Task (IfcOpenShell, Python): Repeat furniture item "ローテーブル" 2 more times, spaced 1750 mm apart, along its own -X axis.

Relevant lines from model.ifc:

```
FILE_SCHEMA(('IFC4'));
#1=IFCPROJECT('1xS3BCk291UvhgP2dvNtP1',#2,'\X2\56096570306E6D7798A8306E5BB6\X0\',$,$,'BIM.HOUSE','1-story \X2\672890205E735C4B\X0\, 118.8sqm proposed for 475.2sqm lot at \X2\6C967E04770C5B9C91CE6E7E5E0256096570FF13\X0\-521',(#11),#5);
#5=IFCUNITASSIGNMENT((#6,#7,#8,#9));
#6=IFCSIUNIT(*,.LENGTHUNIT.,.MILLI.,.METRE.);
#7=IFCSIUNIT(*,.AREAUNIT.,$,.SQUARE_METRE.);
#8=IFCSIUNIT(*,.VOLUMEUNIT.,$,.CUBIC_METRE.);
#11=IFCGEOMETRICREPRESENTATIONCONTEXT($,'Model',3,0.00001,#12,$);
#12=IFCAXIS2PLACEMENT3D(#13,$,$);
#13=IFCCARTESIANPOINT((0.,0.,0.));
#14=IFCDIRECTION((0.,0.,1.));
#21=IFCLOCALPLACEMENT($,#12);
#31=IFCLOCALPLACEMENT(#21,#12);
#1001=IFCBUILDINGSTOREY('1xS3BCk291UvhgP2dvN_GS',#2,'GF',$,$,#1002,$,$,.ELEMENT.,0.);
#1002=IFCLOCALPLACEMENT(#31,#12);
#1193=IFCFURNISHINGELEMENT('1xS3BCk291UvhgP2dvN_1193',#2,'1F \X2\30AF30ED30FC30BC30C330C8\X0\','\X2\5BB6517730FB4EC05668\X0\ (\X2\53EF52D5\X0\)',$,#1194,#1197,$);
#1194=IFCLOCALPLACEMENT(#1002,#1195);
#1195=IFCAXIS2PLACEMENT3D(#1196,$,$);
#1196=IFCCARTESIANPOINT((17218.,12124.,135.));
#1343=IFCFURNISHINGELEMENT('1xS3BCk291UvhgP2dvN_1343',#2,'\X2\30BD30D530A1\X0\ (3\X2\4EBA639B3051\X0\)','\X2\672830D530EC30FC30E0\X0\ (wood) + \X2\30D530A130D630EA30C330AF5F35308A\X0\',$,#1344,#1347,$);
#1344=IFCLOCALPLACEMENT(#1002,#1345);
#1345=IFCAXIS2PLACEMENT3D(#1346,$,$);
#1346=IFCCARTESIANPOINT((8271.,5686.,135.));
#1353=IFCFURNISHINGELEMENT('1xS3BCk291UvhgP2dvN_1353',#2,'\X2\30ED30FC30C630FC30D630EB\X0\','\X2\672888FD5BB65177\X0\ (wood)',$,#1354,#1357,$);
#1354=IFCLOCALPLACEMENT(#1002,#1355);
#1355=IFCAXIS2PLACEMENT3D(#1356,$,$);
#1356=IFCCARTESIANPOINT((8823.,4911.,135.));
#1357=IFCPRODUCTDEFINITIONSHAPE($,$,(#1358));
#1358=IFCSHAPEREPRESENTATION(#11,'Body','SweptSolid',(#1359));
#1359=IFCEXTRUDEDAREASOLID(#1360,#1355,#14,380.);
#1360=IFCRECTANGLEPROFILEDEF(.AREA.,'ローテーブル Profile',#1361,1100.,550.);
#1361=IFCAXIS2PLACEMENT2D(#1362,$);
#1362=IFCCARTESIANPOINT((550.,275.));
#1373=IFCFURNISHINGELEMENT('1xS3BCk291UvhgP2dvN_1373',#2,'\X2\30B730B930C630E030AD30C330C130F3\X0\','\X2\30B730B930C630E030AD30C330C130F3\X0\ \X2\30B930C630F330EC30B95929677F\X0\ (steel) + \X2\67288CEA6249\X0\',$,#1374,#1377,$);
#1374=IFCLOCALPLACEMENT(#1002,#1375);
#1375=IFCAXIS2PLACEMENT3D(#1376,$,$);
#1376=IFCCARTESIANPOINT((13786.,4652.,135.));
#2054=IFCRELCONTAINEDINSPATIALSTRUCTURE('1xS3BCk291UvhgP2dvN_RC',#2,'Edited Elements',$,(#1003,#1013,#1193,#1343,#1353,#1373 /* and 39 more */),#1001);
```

```python
import ifcopenshell
import ifcopenshell.api.geometry
import ifcopenshell.api.root
import ifcopenshell.util.element
import ifcopenshell.util.placement
import ifcopenshell.util.unit

model = ifcopenshell.open("model.ifc")
unit_scale = ifcopenshell.util.unit.calculate_unit_scale(model)


def reuse_history(source, copy):
    """copy_class also copies each property set's owner history, people and application; keep the originals."""
    for rel in copy.IsDefinedBy:
        if rel.is_a("IfcRelDefinesByProperties") and (history := rel.RelatingPropertyDefinition.OwnerHistory):
            rel.RelatingPropertyDefinition.OwnerHistory = source.OwnerHistory
            ifcopenshell.util.element.remove_deep2(model, history)


source = model.by_id(1353)
base = ifcopenshell.util.placement.get_local_placement(source.ObjectPlacement)
step = -base[:3, 0] * 1.75 / unit_scale

for i in range(1, 3):
    copy = ifcopenshell.api.root.copy_class(model, product=source)
    copy.Representation = ifcopenshell.util.element.copy_deep(
        model, source.Representation, exclude=["IfcGeometricRepresentationContext", "IfcRepresentationMap"]
    )
    reuse_history(source, copy)
    matrix = base.copy()
    matrix[:3, 3] += i * step
    print("added at", matrix[:3, 3].round(3) + 0.0)
    ifcopenshell.api.geometry.edit_object_placement(model, product=copy, matrix=matrix, is_si=False)

model.write("model_updated.ifc")
```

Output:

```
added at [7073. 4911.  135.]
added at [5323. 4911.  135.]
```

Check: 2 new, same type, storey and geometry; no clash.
